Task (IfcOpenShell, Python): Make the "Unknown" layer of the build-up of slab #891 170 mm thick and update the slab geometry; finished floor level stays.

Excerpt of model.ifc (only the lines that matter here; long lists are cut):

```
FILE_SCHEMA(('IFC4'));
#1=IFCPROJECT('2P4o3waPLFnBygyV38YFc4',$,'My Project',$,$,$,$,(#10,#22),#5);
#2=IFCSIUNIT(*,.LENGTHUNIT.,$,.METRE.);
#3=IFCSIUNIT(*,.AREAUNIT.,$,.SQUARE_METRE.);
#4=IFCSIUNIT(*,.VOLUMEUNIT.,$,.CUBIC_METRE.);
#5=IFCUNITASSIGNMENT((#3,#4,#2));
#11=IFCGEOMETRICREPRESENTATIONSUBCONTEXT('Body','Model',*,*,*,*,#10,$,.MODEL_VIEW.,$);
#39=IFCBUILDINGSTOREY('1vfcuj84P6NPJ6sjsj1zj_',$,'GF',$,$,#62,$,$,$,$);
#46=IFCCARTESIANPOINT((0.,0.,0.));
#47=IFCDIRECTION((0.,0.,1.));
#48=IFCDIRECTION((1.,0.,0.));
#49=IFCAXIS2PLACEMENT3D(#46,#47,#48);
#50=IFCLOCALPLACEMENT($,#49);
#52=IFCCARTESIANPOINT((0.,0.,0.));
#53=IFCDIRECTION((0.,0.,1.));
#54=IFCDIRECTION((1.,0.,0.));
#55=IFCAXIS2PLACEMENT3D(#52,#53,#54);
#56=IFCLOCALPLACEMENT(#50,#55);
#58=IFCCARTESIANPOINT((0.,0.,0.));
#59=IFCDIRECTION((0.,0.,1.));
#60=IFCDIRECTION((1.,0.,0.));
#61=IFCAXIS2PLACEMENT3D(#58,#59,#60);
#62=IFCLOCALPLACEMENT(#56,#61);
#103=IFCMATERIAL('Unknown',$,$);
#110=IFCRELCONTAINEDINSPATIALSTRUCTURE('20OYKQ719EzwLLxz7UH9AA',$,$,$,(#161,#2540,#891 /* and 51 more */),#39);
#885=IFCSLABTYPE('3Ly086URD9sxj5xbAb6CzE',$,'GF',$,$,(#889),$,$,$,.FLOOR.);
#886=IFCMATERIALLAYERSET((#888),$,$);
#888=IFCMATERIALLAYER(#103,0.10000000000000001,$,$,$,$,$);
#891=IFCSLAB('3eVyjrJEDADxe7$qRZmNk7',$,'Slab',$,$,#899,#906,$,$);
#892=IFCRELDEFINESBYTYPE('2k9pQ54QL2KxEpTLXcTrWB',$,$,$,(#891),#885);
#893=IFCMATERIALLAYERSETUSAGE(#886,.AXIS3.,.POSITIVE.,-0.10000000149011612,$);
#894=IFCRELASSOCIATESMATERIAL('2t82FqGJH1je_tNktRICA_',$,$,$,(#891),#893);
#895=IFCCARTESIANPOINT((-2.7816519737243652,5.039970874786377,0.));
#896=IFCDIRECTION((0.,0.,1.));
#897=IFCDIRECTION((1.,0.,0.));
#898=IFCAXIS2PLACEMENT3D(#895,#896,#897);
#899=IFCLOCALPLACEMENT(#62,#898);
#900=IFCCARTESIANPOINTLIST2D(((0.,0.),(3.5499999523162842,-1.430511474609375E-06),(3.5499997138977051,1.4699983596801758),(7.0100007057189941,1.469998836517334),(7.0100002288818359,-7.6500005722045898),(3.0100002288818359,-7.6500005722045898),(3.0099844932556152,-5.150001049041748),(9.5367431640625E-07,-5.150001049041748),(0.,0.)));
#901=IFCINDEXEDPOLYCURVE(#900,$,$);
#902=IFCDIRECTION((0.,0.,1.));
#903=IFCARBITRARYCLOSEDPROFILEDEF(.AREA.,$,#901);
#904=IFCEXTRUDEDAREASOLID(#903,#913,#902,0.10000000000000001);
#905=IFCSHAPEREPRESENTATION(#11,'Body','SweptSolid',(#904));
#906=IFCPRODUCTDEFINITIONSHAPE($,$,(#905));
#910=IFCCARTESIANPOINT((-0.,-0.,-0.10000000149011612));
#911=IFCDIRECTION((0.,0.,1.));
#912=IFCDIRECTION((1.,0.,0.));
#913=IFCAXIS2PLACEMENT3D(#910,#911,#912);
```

```python
import ifcopenshell
import ifcopenshell.util.element
import ifcopenshell.util.representation
import ifcopenshell.util.unit

model = ifcopenshell.open("model.ifc")
unit_scale = ifcopenshell.util.unit.calculate_unit_scale(model)

layer_set = model.by_id(886)
layer = next(l for l in layer_set.MaterialLayers if l.Material and l.Material.Name == "Unknown")
change = 0.17 / unit_scale - layer.LayerThickness
layer.LayerThickness += change

# Geometry does not follow the layer set by itself.
slabs = [e for e in ifcopenshell.util.element.get_elements_by_material(model, layer_set) if e.is_a("IfcSlab")]
for slab in sorted(slabs, key=lambda e: e.id()):
    body = ifcopenshell.util.representation.get_representation(slab, "Model", "Body")
    solid = body.Items[0]
    old_depth = solid.Depth
    solid.Depth += change
    # Extruded upwards: lower the start of the extrusion so the top stays.
    x, y, z = solid.Position.Location.Coordinates
    solid.Position.Location = model.createIfcCartesianPoint((x, y, z - change))
    print(slab.id(), f"{old_depth:g} -> {solid.Depth:g}")

# The layers are counted up from the underside, which has moved.
for usage in {ifcopenshell.util.element.get_material(slab) for slab in slabs}:
    usage.OffsetFromReferenceLine -= change

model.write("model_updated.ifc")
```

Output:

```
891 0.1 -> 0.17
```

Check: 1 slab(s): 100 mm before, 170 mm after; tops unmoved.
